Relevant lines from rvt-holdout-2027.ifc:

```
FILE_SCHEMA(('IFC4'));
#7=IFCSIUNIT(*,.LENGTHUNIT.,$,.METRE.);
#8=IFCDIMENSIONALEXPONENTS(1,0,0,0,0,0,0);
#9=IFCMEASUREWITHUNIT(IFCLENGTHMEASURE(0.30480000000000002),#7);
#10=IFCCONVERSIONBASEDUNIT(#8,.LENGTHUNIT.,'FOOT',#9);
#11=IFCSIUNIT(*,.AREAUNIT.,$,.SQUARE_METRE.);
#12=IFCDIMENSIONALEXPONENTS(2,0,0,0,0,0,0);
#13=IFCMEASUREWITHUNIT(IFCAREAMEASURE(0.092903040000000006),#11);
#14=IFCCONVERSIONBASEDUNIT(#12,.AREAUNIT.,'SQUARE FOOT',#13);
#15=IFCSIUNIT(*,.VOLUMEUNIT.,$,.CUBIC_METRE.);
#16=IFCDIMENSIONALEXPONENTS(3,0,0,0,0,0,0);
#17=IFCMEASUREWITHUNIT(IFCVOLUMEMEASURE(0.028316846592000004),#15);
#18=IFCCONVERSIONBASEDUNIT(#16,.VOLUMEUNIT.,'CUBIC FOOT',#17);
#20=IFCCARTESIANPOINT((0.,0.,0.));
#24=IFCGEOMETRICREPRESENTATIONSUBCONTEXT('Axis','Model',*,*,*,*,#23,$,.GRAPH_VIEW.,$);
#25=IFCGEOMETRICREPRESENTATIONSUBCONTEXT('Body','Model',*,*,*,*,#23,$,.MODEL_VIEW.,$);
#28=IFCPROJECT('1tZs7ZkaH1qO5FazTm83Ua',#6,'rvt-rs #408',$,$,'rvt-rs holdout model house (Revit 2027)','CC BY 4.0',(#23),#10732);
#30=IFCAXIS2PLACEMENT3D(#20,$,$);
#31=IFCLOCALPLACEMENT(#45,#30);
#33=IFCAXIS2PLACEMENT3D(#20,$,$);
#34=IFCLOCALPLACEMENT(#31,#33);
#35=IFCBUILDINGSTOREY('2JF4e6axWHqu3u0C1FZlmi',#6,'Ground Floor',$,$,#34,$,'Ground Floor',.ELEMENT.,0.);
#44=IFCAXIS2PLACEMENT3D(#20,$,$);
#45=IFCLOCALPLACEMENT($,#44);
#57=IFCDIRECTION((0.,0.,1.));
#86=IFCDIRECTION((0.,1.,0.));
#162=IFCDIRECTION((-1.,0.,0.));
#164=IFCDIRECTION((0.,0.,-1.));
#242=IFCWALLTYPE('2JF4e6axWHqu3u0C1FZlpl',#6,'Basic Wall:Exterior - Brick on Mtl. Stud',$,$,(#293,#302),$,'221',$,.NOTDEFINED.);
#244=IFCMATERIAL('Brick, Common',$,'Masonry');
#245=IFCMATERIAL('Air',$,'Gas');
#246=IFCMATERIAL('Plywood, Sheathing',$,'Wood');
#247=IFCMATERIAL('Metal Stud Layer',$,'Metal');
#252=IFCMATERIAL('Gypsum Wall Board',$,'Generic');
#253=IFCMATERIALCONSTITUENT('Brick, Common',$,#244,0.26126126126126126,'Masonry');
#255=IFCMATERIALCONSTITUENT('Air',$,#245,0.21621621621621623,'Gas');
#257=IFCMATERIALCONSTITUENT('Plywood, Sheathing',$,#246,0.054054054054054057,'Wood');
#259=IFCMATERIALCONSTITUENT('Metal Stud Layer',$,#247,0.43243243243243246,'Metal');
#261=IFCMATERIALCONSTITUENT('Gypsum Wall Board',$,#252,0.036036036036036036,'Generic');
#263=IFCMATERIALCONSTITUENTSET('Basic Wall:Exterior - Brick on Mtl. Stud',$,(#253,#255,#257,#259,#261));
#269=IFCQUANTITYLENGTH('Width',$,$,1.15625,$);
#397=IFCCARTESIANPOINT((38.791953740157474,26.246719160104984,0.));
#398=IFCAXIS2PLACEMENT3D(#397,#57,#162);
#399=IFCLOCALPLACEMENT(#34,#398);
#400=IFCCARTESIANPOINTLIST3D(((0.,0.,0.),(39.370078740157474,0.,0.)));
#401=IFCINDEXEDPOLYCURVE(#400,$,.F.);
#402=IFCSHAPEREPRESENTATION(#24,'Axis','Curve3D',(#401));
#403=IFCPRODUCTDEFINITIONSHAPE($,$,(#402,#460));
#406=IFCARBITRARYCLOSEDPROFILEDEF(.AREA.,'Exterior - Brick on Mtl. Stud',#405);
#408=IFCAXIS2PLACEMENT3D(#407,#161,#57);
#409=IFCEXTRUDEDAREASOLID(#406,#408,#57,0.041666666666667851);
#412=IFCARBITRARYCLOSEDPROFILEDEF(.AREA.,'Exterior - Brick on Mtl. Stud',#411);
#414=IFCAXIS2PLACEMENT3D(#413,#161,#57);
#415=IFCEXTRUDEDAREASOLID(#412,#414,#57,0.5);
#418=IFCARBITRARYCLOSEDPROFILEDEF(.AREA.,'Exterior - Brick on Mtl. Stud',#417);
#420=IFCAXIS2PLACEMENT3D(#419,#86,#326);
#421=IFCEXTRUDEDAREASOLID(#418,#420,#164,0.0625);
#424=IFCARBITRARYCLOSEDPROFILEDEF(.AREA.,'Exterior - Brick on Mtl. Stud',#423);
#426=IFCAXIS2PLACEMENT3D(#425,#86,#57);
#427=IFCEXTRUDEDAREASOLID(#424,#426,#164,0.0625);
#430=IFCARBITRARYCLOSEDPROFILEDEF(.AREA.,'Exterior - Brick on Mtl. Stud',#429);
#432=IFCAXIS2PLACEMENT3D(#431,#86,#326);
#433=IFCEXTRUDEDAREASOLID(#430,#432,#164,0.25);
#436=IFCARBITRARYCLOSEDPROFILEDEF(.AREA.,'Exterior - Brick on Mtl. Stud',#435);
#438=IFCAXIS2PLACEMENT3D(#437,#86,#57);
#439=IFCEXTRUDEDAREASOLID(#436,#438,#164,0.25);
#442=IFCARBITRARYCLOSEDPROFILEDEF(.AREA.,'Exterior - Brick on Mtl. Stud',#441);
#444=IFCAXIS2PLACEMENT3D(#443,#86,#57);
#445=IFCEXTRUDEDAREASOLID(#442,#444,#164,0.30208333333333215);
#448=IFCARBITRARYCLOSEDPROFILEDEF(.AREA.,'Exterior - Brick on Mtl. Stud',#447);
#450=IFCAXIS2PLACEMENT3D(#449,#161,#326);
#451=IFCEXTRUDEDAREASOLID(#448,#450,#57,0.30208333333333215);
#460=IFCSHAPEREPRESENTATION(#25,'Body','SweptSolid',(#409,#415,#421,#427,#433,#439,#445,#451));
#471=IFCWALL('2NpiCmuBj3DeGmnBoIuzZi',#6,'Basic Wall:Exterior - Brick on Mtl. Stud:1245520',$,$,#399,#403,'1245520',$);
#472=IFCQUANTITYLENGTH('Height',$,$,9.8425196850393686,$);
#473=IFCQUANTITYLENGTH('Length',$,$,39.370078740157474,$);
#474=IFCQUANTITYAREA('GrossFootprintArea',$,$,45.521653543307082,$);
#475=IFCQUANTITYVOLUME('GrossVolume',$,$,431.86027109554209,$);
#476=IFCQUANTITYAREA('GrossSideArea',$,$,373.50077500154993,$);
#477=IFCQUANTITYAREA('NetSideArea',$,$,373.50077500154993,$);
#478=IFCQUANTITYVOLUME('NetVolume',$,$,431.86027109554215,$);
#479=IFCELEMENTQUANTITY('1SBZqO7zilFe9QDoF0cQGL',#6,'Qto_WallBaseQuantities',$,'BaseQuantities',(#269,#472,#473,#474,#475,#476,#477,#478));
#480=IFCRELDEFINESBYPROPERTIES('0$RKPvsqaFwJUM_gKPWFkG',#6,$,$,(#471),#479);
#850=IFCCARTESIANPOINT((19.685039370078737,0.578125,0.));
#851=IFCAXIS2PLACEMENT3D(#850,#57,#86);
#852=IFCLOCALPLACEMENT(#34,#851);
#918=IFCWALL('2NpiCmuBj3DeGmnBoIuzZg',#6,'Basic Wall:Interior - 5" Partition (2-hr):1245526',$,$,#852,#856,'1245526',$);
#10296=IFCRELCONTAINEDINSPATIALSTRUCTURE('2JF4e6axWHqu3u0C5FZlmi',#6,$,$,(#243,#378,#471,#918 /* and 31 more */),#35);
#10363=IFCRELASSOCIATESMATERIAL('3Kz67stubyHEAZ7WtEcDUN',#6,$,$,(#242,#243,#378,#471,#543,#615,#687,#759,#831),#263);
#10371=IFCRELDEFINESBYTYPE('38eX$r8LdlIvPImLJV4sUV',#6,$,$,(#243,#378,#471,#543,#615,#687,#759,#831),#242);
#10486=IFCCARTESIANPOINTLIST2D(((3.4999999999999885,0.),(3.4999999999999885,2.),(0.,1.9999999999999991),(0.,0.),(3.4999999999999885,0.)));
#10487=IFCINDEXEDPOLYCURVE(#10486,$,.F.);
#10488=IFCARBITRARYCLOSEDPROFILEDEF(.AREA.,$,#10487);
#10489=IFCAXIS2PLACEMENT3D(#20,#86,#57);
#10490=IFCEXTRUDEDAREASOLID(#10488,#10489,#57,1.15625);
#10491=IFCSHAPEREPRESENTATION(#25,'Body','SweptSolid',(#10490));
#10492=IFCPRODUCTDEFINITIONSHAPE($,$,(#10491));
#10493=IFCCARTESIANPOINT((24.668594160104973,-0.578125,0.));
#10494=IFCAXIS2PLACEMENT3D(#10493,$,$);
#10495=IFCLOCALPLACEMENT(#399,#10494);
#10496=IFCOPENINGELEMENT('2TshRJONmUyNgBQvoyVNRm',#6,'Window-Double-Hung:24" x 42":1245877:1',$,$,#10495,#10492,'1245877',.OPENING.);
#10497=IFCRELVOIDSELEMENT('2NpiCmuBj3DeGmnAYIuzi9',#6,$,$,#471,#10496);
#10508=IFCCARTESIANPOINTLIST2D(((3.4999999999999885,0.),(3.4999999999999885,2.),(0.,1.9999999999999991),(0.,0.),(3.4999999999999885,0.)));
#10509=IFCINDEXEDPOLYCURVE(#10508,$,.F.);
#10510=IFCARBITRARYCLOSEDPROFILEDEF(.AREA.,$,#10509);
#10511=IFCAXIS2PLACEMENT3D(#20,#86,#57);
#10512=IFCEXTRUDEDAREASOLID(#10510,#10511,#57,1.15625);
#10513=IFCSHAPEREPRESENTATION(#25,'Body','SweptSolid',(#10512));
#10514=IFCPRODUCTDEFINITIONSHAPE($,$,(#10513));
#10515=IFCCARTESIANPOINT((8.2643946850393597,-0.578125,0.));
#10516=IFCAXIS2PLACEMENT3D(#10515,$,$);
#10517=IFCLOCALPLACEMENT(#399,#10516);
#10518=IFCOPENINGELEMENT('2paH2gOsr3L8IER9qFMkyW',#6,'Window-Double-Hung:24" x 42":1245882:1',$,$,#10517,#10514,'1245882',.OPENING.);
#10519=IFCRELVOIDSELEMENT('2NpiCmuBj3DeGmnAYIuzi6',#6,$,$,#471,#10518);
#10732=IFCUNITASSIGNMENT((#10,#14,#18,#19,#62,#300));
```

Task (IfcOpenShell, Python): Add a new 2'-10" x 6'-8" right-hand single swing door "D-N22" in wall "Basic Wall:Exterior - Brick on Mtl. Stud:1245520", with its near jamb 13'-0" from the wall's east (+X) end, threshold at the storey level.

```python
import numpy as np
import ifcopenshell
import ifcopenshell.api.feature
import ifcopenshell.api.geometry
import ifcopenshell.api.pset
import ifcopenshell.api.root
import ifcopenshell.api.spatial
import ifcopenshell.geom
import ifcopenshell.util.element
import ifcopenshell.util.placement
import ifcopenshell.util.representation
import ifcopenshell.util.shape
import ifcopenshell.util.unit

model = ifcopenshell.open("rvt-holdout-2027.ifc")
unit_scale = ifcopenshell.util.unit.calculate_unit_scale(model)
area_scale = ifcopenshell.util.unit.calculate_unit_scale(model, "AREAUNIT")
volume_scale = ifcopenshell.util.unit.calculate_unit_scale(model, "VOLUMEUNIT")
settings = ifcopenshell.geom.settings()


def volume(element):
    """Net volume in cubic metres, openings subtracted."""
    shape = ifcopenshell.geom.create_shape(settings, element)
    return ifcopenshell.util.shape.get_volume(shape.geometry)


wall = model.by_id(471)
storey = ifcopenshell.util.element.get_container(wall, ifc_class="IfcBuildingStorey")
context = ifcopenshell.util.representation.get_context(model, "Model", "Body", "MODEL_VIEW")
before = volume(wall)

width, height, from_end, sill = 0.8636, 2.032, 3.9624, 0.0  # metres

# The wall runs along its own X axis, and the end named is its -X end.
wall_shape = ifcopenshell.geom.create_shape(settings, wall)
x, y, z = ifcopenshell.util.shape.get_vertices(wall_shape.geometry).T
start = x.min() + from_end
face, thickness = float(y.min()), float(y.max() - y.min())
wall_matrix = ifcopenshell.util.placement.get_local_placement(wall.ObjectPlacement)
level = ifcopenshell.util.placement.get_local_placement(storey.ObjectPlacement)[2, 3]


def in_wall(x, y):
    """Placement at x, y metres in the wall's axes, at sill height."""
    matrix = wall_matrix.copy()
    matrix[:, 3] = wall_matrix @ np.array([x / unit_scale, y / unit_scale, 0.0, 1.0])
    matrix[2, 3] = level + sill / unit_scale
    return matrix


# Opening: a box that overshoots both wall faces by 50 mm.
opening = ifcopenshell.api.root.create_entity(model, ifc_class="IfcOpeningElement", predefined_type="OPENING")
box = ifcopenshell.api.geometry.add_wall_representation(
    model, context=context, length=width, height=height, thickness=thickness + 0.1
)
ifcopenshell.api.geometry.assign_representation(model, product=opening, representation=box)
ifcopenshell.api.geometry.edit_object_placement(model, product=opening, matrix=in_wall(start, face - 0.05), is_si=False)
ifcopenshell.api.feature.add_feature(model, feature=opening, element=wall)

door = ifcopenshell.api.root.create_entity(model, ifc_class="IfcDoor", name="D-N22", predefined_type="DOOR")
door.OverallWidth, door.OverallHeight = width / unit_scale, height / unit_scale
door.OperationType = "SINGLE_SWING_RIGHT"
body = ifcopenshell.api.geometry.add_door_representation(
    model,
    context=context,
    overall_width=door.OverallWidth,
    overall_height=door.OverallHeight,
    operation_type="SINGLE_SWING_RIGHT",
    lining_properties={"LiningDepth": thickness / unit_scale, "ThresholdDepth": thickness / unit_scale},
)
ifcopenshell.api.geometry.assign_representation(model, product=door, representation=body)
ifcopenshell.api.spatial.assign_container(model, products=[door], relating_structure=storey)
ifcopenshell.api.feature.add_filling(model, opening=opening, element=door)

# The lining spans the wall, so the door starts at the wall face.
ifcopenshell.api.geometry.edit_object_placement(model, product=door, matrix=in_wall(start, face), is_si=False)

after = volume(wall)

# Update the wall's stored quantities.
qto = model.by_id(ifcopenshell.util.element.get_pset(wall, "Qto_WallBaseQuantities", should_inherit=False)["id"])
ifcopenshell.api.pset.edit_qto(model, qto=qto, properties={
    "NetSideArea": after / thickness / area_scale,
    "NetVolume": after / volume_scale,
})

print(f"wall volume {before:.3f} -> {after:.3f} m3")

model.write("rvt-holdout-2027_edited.ifc")
```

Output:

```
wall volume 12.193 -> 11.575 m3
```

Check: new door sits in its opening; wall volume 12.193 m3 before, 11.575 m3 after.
